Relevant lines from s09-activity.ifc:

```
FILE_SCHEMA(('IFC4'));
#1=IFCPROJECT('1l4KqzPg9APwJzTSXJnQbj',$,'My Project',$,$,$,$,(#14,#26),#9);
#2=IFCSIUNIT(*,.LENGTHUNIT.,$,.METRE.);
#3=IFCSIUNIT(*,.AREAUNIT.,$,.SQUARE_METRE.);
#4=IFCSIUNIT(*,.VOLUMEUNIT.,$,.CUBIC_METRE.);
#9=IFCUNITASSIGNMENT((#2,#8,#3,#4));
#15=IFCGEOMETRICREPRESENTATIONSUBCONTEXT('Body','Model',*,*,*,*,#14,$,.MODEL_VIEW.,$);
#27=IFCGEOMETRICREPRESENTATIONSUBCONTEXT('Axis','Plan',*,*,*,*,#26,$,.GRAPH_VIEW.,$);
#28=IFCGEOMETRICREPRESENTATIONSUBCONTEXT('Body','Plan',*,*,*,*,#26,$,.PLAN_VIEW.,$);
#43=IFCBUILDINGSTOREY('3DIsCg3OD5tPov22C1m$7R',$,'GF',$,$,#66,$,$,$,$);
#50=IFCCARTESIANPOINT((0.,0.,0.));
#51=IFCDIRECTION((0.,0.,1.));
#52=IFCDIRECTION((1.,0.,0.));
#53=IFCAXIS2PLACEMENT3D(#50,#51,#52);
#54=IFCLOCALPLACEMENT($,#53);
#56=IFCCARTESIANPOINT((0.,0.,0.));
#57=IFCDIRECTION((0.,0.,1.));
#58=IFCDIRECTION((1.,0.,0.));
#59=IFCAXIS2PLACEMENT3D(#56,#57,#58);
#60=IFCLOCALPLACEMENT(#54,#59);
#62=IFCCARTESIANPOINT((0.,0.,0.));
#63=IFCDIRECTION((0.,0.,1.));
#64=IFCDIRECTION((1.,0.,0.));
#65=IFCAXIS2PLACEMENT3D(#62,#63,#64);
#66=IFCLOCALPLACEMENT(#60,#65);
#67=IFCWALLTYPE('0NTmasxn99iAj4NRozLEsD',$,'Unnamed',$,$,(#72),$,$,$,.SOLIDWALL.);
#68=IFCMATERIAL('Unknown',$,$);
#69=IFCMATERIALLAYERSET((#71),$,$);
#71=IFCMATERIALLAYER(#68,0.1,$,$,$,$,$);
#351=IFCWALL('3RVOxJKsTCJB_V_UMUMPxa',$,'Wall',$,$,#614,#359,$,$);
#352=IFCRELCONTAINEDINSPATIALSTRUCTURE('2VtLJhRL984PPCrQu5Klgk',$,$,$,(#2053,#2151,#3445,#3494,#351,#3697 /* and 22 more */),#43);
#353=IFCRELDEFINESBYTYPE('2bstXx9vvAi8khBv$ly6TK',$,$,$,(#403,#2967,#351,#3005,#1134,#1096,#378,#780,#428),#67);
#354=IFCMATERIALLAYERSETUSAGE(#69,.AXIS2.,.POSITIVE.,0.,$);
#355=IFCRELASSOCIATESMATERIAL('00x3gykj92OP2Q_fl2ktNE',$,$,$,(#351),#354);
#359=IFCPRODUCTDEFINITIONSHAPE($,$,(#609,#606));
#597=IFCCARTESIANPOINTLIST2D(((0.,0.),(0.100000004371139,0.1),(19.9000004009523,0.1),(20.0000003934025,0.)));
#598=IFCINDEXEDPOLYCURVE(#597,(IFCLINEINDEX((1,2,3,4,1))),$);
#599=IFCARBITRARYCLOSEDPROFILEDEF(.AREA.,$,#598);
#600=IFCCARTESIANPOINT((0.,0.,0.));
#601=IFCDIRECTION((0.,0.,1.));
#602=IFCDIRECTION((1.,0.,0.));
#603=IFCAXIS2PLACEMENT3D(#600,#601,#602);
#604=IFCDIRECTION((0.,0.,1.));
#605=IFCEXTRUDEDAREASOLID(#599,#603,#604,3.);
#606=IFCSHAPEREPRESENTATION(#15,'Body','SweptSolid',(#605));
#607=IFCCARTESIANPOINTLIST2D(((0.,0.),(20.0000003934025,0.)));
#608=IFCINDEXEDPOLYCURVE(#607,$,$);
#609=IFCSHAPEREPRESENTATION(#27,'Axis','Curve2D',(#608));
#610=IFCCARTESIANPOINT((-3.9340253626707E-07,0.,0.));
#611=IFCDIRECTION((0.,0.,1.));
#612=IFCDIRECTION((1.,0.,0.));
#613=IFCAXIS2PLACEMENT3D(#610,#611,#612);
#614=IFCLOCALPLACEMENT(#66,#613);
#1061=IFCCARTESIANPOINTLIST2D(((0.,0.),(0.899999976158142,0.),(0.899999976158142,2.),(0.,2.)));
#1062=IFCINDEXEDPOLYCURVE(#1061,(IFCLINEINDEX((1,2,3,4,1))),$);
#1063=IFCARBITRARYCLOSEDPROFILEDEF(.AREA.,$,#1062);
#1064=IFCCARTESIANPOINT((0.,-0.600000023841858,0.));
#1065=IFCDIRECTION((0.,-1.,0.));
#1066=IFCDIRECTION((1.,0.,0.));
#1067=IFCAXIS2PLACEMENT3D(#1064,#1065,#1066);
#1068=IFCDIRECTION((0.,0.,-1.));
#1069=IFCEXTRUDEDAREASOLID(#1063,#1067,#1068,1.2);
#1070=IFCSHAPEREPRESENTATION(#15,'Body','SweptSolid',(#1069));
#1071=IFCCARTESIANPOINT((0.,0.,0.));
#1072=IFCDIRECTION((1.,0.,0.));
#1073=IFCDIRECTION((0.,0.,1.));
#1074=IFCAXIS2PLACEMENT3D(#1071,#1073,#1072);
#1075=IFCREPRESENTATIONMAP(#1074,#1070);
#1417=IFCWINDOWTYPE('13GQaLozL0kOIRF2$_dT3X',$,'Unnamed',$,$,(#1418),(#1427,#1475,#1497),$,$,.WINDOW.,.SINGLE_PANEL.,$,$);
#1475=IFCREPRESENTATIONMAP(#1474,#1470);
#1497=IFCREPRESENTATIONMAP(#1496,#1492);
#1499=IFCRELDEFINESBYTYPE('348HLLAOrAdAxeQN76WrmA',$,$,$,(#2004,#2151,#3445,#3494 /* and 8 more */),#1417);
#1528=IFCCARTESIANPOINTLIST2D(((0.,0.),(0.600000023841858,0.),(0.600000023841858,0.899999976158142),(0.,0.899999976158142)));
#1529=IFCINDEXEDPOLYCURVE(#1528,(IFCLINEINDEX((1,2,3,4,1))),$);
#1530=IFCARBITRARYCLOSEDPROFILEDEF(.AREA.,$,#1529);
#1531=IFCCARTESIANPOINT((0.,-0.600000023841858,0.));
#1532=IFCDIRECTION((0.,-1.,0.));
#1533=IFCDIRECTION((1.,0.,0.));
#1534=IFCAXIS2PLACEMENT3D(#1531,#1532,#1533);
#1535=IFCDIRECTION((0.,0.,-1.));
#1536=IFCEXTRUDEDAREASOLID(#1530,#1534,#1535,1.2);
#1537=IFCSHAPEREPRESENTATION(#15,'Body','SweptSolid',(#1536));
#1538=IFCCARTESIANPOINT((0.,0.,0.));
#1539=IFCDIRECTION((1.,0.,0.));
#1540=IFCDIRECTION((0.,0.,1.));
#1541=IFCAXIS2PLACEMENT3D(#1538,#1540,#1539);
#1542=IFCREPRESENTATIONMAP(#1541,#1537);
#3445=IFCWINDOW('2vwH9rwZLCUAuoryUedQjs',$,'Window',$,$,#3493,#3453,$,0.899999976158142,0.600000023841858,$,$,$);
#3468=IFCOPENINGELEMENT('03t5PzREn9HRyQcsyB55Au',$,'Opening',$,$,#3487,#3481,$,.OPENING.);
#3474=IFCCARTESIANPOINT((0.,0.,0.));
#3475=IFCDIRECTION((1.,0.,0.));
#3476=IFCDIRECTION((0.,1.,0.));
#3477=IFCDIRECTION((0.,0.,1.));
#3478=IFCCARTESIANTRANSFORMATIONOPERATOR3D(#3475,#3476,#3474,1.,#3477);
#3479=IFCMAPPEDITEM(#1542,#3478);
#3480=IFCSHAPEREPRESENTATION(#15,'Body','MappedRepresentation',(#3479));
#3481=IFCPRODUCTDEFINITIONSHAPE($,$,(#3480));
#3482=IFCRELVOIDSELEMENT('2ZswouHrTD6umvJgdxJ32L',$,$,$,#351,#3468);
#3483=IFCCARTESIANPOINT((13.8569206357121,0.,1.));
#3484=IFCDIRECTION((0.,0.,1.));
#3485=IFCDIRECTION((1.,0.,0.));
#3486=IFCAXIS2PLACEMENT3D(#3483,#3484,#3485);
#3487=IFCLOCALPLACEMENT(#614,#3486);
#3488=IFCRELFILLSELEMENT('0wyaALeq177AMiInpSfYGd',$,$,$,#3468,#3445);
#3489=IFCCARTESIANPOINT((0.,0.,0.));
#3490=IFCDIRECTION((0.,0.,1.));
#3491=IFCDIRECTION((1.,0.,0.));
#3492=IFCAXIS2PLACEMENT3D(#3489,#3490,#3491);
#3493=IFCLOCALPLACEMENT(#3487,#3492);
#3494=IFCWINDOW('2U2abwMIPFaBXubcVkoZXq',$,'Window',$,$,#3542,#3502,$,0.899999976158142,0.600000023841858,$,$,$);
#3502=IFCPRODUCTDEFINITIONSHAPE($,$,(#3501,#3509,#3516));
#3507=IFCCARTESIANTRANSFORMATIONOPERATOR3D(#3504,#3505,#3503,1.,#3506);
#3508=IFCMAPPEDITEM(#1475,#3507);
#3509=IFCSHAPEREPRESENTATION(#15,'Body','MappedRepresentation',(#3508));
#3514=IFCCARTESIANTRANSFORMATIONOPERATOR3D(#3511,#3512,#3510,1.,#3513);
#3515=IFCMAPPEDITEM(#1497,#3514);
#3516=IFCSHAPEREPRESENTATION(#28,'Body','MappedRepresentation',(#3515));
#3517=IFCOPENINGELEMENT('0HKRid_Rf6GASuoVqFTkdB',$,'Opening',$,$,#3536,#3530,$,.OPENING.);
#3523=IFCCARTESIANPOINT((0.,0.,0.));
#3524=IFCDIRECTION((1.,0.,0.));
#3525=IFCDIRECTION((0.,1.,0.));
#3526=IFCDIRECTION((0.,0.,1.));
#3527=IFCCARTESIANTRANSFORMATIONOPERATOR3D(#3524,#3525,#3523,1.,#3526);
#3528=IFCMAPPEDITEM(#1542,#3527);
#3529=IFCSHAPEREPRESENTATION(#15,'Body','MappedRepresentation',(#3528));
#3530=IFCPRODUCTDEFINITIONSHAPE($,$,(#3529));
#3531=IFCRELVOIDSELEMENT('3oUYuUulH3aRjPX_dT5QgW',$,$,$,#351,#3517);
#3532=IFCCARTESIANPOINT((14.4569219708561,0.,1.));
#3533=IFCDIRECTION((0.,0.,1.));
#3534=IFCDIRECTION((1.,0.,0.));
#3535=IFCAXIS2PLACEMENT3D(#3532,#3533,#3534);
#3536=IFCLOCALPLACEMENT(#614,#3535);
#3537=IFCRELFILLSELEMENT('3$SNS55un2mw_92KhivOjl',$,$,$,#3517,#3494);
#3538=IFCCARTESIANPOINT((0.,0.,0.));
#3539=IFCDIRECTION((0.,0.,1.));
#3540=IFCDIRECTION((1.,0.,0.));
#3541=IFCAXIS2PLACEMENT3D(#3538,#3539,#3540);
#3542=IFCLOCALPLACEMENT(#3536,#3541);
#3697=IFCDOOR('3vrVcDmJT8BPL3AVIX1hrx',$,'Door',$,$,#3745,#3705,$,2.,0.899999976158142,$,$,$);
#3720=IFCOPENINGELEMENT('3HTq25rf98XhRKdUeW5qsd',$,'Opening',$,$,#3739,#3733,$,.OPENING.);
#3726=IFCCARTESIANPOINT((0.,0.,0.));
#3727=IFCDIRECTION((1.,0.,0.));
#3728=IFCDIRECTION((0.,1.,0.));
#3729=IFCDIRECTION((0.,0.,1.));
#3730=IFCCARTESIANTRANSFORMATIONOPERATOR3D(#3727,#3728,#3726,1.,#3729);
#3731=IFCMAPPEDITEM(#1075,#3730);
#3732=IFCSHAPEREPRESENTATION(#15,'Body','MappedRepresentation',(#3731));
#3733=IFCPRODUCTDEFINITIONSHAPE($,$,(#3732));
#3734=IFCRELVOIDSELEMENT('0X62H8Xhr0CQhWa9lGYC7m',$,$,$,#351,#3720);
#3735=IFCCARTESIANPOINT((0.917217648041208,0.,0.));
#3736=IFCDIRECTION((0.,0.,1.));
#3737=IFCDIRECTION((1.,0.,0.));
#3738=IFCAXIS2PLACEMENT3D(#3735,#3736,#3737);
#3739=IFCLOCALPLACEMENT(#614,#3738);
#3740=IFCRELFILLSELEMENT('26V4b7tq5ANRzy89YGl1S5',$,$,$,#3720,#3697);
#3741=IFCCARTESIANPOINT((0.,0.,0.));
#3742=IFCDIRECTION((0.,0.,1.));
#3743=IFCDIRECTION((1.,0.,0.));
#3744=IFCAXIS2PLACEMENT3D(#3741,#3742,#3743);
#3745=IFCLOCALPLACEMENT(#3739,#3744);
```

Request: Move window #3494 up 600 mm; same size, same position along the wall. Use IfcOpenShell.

```python
import numpy as np
import ifcopenshell
import ifcopenshell.api.geometry
import ifcopenshell.util.placement
import ifcopenshell.util.unit

model = ifcopenshell.open("s09-activity.ifc")
unit_scale = ifcopenshell.util.unit.calculate_unit_scale(model)

window = model.by_guid("2U2abwMIPFaBXubcVkoZXq")
opening = window.FillsVoids[0].RelatingOpeningElement
dz = 0.6 / unit_scale

shift = np.array([0.0, 0.0, dz])
# The window is placed relative to its opening, so it follows when the opening moves.
matrix = ifcopenshell.util.placement.get_local_placement(opening.ObjectPlacement)
matrix[:3, 3] += shift
ifcopenshell.api.geometry.edit_object_placement(
    model, product=opening, matrix=matrix, is_si=False, should_transform_children=True
)

print(f"moved by {dz * unit_scale:+.3f} m")

model.write("s09-activity_v2.ifc")
```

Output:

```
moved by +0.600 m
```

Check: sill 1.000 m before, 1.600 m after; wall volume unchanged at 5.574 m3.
